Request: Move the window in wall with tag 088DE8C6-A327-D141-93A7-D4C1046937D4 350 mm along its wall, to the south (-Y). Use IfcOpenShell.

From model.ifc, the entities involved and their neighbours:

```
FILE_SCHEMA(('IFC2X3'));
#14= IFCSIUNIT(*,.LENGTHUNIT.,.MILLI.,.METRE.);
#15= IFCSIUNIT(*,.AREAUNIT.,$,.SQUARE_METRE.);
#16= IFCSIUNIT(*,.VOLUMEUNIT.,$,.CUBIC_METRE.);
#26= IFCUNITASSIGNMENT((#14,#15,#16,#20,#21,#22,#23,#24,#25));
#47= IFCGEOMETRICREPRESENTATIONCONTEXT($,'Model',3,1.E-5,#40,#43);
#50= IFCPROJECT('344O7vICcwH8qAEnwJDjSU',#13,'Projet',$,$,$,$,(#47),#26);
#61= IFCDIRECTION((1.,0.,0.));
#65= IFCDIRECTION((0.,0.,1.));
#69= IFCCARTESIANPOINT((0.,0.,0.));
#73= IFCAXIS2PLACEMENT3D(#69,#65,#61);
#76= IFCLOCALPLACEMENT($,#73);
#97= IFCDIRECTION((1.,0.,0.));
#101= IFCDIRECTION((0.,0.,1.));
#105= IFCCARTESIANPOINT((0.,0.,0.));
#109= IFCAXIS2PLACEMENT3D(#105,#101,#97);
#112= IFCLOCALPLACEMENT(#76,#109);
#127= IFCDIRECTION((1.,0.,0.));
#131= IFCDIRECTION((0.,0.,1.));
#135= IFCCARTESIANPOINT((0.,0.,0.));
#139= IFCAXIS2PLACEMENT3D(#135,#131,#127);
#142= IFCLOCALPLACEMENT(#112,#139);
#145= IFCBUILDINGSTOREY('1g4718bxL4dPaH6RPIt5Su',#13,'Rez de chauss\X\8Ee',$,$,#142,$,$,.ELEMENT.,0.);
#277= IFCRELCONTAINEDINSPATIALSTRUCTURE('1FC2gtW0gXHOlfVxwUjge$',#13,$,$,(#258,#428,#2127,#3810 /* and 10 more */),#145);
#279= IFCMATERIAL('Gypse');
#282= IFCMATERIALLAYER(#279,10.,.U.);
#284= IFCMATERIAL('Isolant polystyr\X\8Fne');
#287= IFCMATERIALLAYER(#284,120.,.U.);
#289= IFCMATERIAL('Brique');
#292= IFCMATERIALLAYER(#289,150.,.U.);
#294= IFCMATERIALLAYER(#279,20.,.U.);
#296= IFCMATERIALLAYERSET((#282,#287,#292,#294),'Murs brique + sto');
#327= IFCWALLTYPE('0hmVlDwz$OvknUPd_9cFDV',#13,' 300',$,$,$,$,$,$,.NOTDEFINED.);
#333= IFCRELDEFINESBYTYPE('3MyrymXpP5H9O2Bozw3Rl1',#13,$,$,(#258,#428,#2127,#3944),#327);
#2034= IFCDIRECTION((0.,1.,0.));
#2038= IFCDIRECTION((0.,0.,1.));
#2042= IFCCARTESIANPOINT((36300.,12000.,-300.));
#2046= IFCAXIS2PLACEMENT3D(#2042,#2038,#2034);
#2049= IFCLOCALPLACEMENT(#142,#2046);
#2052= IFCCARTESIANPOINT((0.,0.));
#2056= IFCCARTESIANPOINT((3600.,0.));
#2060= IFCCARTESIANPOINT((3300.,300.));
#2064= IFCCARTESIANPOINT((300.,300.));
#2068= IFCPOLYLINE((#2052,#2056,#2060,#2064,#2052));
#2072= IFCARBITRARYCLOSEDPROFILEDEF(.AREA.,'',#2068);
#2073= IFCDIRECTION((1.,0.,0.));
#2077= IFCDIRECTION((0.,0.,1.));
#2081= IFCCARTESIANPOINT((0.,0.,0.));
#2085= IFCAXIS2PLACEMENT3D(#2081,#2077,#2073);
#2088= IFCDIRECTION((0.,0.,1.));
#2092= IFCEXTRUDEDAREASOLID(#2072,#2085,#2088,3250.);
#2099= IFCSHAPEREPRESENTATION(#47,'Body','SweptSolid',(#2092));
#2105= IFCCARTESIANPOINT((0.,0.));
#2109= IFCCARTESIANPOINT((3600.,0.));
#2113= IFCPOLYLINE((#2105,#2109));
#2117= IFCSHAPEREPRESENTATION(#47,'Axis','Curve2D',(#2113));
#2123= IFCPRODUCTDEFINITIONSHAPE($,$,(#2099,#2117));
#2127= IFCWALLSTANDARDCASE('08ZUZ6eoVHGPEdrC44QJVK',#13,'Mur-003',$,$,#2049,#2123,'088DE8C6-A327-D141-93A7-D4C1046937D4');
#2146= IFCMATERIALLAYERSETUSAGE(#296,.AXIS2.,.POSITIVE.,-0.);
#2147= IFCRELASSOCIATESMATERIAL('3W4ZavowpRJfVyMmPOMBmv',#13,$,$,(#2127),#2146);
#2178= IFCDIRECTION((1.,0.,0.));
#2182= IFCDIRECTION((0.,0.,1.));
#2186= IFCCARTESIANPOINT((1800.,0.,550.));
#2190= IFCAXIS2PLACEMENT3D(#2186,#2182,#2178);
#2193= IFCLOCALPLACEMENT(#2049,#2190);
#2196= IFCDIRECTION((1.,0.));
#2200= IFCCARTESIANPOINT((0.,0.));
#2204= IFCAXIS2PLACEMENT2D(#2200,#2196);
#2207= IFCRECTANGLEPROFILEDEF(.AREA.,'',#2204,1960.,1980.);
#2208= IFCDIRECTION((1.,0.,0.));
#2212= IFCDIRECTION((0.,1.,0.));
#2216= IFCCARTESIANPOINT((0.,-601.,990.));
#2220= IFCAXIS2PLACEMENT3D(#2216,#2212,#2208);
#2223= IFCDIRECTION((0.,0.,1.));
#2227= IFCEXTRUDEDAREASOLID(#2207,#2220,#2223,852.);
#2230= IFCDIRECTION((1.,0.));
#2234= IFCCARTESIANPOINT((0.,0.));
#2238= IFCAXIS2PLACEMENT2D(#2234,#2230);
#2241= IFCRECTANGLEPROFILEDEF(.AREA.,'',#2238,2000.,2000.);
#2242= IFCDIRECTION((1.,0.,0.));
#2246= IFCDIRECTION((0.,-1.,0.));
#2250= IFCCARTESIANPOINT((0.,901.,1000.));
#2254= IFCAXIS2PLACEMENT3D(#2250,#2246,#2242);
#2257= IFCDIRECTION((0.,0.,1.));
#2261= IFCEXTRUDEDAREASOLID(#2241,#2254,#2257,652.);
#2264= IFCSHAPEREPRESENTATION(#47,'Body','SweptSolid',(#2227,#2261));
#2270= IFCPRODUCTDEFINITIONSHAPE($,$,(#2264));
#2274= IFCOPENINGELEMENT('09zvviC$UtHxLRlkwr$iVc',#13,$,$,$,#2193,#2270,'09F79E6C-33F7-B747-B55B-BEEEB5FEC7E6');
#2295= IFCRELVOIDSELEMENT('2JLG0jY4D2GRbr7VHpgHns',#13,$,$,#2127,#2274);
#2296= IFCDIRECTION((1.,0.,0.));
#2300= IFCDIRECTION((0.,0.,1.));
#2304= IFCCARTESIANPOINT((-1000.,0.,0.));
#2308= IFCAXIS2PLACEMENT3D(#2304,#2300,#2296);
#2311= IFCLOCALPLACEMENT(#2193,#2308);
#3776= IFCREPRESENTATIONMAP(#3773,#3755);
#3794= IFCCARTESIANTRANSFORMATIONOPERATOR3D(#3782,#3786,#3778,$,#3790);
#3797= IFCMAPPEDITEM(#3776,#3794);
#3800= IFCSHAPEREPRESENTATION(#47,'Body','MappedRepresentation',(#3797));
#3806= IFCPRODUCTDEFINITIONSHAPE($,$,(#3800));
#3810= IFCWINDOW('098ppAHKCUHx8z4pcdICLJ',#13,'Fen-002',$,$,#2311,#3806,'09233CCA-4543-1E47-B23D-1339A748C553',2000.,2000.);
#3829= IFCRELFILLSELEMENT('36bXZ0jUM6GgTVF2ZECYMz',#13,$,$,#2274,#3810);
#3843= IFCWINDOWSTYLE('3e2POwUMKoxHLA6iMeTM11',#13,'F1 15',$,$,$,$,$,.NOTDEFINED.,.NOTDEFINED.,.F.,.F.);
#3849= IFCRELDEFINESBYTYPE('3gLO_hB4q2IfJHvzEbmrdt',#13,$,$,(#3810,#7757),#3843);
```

```python
import ifcopenshell
import ifcopenshell.api.geometry
import ifcopenshell.util.placement

model = ifcopenshell.open("model.ifc")

window = model.by_id(3810)
opening = window.FillsVoids[0].RelatingOpeningElement
wall = opening.VoidsElements[0].RelatingBuildingElement

wall_matrix = ifcopenshell.util.placement.get_local_placement(wall.ObjectPlacement)
shift = wall_matrix[:3, 0] * -350.0
before = ifcopenshell.util.placement.get_local_placement(window.ObjectPlacement)[:3, 3].copy()

# The window is placed relative to its opening, so it follows when the opening moves.
matrix = ifcopenshell.util.placement.get_local_placement(opening.ObjectPlacement)
matrix[:3, 3] += shift
ifcopenshell.api.geometry.edit_object_placement(
    model, product=opening, matrix=matrix, is_si=False, should_transform_children=True
)

after = ifcopenshell.util.placement.get_local_placement(window.ObjectPlacement)[:3, 3]
print("window moved by", (after - before).round(3) + 0.0)

model.write("model_updated.ifc")
```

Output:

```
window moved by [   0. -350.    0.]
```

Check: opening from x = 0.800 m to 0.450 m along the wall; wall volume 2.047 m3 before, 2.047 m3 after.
